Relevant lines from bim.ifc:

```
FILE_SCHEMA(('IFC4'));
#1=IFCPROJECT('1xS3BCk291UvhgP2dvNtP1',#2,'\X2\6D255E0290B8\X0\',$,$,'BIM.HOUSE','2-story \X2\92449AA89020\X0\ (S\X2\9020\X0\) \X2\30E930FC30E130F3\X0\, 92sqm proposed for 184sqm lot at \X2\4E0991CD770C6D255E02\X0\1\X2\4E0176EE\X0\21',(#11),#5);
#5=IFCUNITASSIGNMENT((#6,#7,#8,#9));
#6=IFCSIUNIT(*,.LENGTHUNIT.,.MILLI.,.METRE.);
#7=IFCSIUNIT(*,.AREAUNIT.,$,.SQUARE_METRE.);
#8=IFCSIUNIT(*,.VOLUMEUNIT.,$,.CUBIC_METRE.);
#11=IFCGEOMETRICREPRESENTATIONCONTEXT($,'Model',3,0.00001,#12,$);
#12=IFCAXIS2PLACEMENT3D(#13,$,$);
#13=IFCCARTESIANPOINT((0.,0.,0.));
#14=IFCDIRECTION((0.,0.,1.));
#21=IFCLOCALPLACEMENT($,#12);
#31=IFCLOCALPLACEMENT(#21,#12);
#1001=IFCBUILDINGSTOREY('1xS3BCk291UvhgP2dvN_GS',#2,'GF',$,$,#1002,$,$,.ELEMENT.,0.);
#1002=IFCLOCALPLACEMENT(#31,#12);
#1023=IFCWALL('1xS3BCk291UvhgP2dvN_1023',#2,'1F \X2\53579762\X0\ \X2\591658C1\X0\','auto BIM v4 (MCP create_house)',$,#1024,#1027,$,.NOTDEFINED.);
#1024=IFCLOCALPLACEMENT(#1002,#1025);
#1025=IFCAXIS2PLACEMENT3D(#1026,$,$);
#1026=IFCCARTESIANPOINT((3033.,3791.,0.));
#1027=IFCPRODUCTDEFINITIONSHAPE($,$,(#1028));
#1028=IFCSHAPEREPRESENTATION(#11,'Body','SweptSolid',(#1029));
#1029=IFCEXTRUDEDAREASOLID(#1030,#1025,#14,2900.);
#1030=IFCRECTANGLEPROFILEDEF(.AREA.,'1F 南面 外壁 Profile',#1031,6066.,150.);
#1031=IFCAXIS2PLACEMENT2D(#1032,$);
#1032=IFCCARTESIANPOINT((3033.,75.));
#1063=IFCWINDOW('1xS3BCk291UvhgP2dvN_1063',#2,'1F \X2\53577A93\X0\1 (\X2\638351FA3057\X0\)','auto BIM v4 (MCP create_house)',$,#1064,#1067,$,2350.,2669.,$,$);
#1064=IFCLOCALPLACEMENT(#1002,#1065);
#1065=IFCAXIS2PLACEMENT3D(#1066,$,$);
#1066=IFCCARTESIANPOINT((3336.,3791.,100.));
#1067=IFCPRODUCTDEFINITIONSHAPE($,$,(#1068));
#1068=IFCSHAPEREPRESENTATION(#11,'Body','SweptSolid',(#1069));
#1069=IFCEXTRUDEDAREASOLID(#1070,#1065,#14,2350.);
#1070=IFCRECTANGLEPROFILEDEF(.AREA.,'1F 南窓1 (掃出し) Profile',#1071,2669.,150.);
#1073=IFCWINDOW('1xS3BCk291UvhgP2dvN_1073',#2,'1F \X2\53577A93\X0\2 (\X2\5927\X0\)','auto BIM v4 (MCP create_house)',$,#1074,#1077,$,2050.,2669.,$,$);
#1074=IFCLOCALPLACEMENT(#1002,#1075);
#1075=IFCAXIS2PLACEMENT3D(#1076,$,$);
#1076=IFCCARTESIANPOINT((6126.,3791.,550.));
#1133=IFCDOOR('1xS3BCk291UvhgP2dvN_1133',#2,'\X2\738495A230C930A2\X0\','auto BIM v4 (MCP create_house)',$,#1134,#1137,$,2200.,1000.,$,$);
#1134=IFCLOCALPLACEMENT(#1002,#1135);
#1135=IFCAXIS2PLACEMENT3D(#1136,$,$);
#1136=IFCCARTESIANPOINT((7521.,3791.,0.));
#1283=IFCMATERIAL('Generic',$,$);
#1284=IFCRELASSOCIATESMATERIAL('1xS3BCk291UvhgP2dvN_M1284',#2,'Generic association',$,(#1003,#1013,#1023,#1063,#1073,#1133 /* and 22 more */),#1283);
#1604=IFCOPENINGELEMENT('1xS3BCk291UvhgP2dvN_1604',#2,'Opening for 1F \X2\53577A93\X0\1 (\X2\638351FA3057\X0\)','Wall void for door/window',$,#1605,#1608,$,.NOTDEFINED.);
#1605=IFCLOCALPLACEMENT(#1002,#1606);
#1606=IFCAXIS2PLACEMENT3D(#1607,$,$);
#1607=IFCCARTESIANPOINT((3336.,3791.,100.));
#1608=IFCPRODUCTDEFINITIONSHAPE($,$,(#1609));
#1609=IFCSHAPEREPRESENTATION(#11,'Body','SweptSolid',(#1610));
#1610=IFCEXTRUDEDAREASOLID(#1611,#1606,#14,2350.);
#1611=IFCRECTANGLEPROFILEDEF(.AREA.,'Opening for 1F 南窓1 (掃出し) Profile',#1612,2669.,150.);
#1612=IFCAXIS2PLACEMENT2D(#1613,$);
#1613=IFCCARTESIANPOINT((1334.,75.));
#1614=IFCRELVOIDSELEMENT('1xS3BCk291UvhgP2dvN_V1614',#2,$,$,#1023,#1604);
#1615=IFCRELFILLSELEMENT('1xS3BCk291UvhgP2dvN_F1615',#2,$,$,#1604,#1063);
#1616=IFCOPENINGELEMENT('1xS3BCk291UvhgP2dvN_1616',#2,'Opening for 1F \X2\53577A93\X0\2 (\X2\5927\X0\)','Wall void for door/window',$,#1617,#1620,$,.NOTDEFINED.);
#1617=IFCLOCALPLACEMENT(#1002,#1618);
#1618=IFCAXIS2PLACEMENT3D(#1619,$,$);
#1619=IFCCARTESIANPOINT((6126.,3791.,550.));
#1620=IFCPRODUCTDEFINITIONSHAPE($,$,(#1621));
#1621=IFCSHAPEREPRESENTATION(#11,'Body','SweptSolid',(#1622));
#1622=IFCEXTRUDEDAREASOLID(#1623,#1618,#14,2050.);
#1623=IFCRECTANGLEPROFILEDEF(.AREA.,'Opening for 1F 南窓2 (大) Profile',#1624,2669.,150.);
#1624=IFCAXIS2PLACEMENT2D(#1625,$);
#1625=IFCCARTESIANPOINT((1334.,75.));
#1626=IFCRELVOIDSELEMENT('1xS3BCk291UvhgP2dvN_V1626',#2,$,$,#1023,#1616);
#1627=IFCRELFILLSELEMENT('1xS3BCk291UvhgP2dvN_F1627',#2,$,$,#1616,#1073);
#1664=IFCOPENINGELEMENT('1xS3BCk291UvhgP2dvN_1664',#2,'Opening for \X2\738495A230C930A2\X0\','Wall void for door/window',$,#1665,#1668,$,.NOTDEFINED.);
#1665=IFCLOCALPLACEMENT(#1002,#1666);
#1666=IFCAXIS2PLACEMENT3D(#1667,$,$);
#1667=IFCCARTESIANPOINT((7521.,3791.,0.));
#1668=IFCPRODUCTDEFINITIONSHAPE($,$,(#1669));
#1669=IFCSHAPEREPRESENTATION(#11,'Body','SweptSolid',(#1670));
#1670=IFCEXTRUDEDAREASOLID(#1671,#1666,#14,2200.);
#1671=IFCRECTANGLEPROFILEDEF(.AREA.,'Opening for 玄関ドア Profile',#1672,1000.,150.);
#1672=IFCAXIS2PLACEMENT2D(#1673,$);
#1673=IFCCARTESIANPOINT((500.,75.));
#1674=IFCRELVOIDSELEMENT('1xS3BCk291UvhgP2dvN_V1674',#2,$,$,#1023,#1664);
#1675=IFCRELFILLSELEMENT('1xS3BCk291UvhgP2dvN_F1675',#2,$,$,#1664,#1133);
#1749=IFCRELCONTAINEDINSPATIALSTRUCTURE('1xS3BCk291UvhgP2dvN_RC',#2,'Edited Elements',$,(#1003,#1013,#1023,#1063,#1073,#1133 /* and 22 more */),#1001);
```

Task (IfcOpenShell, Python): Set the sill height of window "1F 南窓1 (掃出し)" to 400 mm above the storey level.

```python
import numpy as np
import ifcopenshell
import ifcopenshell.api.geometry
import ifcopenshell.geom
import ifcopenshell.util.element
import ifcopenshell.util.placement
import ifcopenshell.util.shape
import ifcopenshell.util.unit

model = ifcopenshell.open("bim.ifc")
unit_scale = ifcopenshell.util.unit.calculate_unit_scale(model)

window = model.by_id(1063)
opening = window.FillsVoids[0].RelatingOpeningElement
storey = ifcopenshell.util.element.get_container(window, ifc_class="IfcBuildingStorey")
level = ifcopenshell.util.placement.get_local_placement(storey.ObjectPlacement)[2, 3]

# The opening's origin need not be at the sill, so measure its lowest point.
shape = ifcopenshell.geom.create_shape(ifcopenshell.geom.settings(), opening)
bottom = ifcopenshell.util.shape.get_shape_bottom_elevation(shape, shape.geometry) / unit_scale
dz = level + 400.0 - bottom

shift = np.array([0.0, 0.0, dz])
# The window is not placed relative to its opening, so move both.
for product in (opening, window):
    matrix = ifcopenshell.util.placement.get_local_placement(product.ObjectPlacement)
    matrix[:3, 3] += shift
    ifcopenshell.api.geometry.edit_object_placement(model, product=product, matrix=matrix, is_si=False)

print(f"moved by {dz * unit_scale:+.3f} m")

model.write("bim-out.ifc")
```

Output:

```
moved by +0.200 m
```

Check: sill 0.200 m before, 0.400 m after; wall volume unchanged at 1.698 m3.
